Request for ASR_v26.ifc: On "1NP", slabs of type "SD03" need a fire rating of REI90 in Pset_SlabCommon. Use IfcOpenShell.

First a look at what the model holds.

```python
import ifcopenshell
import ifcopenshell.util.element

model = ifcopenshell.open("ASR_v26.ifc")
print(model.schema)
storey = next(s for s in model.by_type("IfcBuildingStorey") if s.Name == "1NP")
slabs = [e for e in ifcopenshell.util.element.get_decomposition(storey) if e.is_a("IfcSlab")]
seen = {}
for e in slabs:
    element_type = ifcopenshell.util.element.get_type(e)
    key = (element_type.Name if element_type != e and element_type else None, ifcopenshell.util.element.get_pset(e, "Pset_SlabCommon", "FireRating"))
    seen[key] = seen.get(key, 0) + 1
for (name, value), count in sorted(seen.items(), key=str):
    print(count, "x", name, "|", value)
```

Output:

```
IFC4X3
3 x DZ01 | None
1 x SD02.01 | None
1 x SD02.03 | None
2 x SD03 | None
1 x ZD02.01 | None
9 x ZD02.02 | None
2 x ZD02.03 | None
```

```python
import ifcopenshell
import ifcopenshell.api.pset
import ifcopenshell.util.element

model = ifcopenshell.open("ASR_v26.ifc")

storey = next(s for s in model.by_type("IfcBuildingStorey") if s.Name == "1NP")
slabs = [e for e in ifcopenshell.util.element.get_decomposition(storey) if e.is_a("IfcSlab")]

count = 0
for e in slabs:
    element_type = ifcopenshell.util.element.get_type(e)
    if element_type in (None, e) or element_type.Name != "SD03":
        continue
    # add_pset returns the element's existing set when there is one.
    pset = ifcopenshell.api.pset.add_pset(model, product=e, name="Pset_SlabCommon")
    ifcopenshell.api.pset.edit_pset(model, pset=pset, properties={"FireRating": "REI90"})
    count += 1

print(count, "slabs updated")

model.write("ASR_v26_updated.ifc")
```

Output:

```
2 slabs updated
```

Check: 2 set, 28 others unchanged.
